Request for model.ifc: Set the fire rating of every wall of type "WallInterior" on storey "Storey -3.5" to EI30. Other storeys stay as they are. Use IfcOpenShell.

First a look at what the model holds.

```python
import ifcopenshell
import ifcopenshell.util.element

model = ifcopenshell.open("model.ifc")
print(model.schema)
storey = next(s for s in model.by_type("IfcBuildingStorey") if s.Name == "Storey -3.5")
walls = [e for e in ifcopenshell.util.element.get_decomposition(storey) if e.is_a("IfcWall")]
seen = {}
for e in walls:
    element_type = ifcopenshell.util.element.get_type(e)
    key = (element_type.Name if element_type != e and element_type else None, ifcopenshell.util.element.get_pset(e, "Pset_WallCommon", "FireRating"))
    seen[key] = seen.get(key, 0) + 1
for (name, value), count in sorted(seen.items(), key=str):
    print(count, "x", name, "|", value)
```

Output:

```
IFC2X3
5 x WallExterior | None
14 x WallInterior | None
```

```python
import ifcopenshell
import ifcopenshell.api.pset
import ifcopenshell.util.element

model = ifcopenshell.open("model.ifc")

storey = next(s for s in model.by_type("IfcBuildingStorey") if s.Name == "Storey -3.5")
walls = [e for e in ifcopenshell.util.element.get_decomposition(storey) if e.is_a("IfcWall")]

count = 0
for e in walls:
    element_type = ifcopenshell.util.element.get_type(e)
    if element_type in (None, e) or element_type.Name != "WallInterior":
        continue
    # add_pset returns the element's existing set when there is one.
    pset = ifcopenshell.api.pset.add_pset(model, product=e, name="Pset_WallCommon")
    ifcopenshell.api.pset.edit_pset(model, pset=pset, properties={"FireRating": "EI30"})
    count += 1

print(count, "walls updated")

model.write("model_rev.ifc")
```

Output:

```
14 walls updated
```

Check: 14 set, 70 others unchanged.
